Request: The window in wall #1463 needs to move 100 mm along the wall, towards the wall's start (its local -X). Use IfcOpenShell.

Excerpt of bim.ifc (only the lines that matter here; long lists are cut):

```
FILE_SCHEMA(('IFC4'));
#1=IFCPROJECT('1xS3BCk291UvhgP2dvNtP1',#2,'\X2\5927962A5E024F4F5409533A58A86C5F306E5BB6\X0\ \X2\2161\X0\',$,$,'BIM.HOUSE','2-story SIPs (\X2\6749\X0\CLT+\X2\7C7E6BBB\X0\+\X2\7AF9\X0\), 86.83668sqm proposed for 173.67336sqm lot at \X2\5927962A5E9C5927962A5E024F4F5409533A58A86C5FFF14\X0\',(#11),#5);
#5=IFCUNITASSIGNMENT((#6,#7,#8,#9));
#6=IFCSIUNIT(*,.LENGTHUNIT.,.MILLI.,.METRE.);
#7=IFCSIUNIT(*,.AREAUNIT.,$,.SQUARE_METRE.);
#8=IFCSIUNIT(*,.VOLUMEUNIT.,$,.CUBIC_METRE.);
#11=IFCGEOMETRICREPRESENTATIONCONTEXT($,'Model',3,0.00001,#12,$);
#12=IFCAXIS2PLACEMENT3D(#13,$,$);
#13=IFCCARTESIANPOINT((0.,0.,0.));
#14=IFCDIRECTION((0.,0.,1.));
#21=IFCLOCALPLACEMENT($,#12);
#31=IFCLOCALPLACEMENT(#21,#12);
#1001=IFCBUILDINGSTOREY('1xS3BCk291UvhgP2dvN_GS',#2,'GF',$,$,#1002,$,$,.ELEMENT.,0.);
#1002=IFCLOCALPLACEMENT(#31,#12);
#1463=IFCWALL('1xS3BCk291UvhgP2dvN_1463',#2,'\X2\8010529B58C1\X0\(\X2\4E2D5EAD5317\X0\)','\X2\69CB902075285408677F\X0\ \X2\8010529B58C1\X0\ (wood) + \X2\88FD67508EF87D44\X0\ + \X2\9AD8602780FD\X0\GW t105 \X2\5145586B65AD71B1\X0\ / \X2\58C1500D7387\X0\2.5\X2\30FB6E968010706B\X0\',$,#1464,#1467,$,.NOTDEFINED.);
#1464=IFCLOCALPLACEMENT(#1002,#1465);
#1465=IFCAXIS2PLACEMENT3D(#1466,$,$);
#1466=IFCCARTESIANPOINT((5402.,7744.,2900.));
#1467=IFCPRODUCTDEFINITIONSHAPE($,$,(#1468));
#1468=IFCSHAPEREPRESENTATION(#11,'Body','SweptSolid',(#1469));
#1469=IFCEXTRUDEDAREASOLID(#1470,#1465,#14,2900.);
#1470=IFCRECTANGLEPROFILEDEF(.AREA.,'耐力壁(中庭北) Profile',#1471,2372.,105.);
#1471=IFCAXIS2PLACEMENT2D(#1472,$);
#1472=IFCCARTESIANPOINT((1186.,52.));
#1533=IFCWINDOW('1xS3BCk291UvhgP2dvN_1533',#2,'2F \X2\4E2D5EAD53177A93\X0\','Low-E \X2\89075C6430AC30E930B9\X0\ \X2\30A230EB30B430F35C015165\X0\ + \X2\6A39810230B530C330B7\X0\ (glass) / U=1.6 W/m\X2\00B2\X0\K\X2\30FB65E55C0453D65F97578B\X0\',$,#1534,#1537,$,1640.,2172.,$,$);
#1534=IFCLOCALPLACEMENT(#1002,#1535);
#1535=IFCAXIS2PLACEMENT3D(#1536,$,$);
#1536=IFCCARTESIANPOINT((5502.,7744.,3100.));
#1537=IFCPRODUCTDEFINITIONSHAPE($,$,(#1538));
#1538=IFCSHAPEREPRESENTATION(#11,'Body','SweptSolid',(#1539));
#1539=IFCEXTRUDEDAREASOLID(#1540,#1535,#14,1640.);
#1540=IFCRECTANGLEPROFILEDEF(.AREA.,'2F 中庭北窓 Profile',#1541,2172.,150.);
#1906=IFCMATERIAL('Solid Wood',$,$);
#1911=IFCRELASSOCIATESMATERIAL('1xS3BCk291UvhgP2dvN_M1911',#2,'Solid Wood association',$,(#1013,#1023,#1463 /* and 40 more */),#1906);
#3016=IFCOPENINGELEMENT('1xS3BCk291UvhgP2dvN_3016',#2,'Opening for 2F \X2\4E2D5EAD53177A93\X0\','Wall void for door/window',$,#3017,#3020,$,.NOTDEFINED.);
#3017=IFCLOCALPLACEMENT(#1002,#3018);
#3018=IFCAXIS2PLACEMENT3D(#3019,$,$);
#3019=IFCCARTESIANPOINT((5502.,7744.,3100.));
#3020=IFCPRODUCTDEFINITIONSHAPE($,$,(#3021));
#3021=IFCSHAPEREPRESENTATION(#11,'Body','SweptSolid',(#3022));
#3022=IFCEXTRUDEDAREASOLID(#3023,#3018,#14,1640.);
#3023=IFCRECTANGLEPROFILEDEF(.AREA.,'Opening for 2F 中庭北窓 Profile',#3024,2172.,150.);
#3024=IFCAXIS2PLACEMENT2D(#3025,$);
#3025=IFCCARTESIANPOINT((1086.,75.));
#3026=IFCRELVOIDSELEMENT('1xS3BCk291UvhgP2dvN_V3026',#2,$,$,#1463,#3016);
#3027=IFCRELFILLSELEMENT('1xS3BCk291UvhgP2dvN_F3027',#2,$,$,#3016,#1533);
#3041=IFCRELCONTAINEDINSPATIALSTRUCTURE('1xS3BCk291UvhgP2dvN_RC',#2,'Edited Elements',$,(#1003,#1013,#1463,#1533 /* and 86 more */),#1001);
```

```python
import ifcopenshell
import ifcopenshell.api.geometry
import ifcopenshell.util.placement

model = ifcopenshell.open("bim.ifc")

window = model.by_guid("1xS3BCk291UvhgP2dvN_1533")
opening = window.FillsVoids[0].RelatingOpeningElement
wall = opening.VoidsElements[0].RelatingBuildingElement

wall_matrix = ifcopenshell.util.placement.get_local_placement(wall.ObjectPlacement)
shift = wall_matrix[:3, 0] * -100.0
before = ifcopenshell.util.placement.get_local_placement(window.ObjectPlacement)[:3, 3].copy()

# The window is not placed relative to its opening, so move both.
for product in (opening, window):
    matrix = ifcopenshell.util.placement.get_local_placement(product.ObjectPlacement)
    matrix[:3, 3] += shift
    ifcopenshell.api.geometry.edit_object_placement(model, product=product, matrix=matrix, is_si=False)

after = ifcopenshell.util.placement.get_local_placement(window.ObjectPlacement)[:3, 3]
print("window moved by", (after - before).round(3) + 0.0)

model.write("bim-out.ifc")
```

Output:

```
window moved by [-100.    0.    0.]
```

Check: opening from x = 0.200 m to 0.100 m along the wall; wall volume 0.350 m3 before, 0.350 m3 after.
